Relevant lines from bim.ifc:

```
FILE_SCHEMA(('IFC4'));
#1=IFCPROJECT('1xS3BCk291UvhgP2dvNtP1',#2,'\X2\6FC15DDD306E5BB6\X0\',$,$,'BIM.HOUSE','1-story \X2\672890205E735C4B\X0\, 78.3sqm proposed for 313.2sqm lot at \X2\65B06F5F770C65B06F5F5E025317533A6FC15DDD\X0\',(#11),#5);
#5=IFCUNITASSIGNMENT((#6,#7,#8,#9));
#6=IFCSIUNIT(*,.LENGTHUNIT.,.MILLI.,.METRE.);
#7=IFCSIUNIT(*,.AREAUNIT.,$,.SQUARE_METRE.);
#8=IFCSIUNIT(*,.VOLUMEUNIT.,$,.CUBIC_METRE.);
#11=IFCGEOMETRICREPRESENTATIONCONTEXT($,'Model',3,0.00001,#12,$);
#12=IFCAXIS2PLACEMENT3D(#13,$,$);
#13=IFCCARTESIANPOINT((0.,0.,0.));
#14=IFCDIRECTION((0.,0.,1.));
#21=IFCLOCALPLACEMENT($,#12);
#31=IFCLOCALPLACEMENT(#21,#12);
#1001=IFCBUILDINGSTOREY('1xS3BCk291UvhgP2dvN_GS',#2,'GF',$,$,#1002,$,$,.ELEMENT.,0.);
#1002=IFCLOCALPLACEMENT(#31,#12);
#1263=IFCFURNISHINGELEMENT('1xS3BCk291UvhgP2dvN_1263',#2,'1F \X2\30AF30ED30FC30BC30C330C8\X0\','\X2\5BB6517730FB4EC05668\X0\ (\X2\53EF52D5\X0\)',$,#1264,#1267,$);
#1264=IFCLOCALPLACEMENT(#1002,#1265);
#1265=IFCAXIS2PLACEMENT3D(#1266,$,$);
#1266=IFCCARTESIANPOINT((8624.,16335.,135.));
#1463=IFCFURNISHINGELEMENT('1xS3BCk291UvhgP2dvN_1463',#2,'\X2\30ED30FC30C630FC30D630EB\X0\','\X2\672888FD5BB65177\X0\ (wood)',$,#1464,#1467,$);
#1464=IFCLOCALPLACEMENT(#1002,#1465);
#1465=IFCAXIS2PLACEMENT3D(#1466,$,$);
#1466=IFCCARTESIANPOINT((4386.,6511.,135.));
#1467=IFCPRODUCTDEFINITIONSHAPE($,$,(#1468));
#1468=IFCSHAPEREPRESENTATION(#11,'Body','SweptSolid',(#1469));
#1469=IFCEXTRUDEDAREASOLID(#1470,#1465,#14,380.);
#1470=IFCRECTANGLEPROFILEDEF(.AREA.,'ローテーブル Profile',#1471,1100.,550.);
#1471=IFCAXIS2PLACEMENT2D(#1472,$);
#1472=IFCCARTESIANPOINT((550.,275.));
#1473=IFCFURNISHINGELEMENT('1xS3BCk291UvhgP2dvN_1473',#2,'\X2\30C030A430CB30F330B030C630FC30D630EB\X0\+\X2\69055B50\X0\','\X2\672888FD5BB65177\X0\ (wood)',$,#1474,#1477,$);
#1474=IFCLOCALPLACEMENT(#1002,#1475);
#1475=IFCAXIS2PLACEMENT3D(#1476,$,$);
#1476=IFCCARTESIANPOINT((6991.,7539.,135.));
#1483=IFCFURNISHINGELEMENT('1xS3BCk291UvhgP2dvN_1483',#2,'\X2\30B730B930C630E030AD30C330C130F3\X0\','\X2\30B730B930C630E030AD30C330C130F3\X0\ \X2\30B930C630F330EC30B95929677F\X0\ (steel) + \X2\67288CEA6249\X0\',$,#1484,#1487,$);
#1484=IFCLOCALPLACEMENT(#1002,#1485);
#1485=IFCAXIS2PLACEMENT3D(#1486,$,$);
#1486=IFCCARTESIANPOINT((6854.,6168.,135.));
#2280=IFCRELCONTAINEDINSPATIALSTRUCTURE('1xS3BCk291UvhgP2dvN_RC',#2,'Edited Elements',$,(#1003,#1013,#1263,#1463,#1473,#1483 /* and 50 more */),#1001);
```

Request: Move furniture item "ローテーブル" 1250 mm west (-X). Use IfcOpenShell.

```python
import ifcopenshell
import ifcopenshell.api.geometry
import ifcopenshell.util.placement

model = ifcopenshell.open("bim.ifc")

item = model.by_id(1463)
matrix = ifcopenshell.util.placement.get_local_placement(item.ObjectPlacement)
matrix[0, 3] -= 1250.0
ifcopenshell.api.geometry.edit_object_placement(model, product=item, matrix=matrix, is_si=False)

print(ifcopenshell.util.placement.get_local_placement(item.ObjectPlacement).round(3) + 0.0)

model.write("bim-out.ifc")
```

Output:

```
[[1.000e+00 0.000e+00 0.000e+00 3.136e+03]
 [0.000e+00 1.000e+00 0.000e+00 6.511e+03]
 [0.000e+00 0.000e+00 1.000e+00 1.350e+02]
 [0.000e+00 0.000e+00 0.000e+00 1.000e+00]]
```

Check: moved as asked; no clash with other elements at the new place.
